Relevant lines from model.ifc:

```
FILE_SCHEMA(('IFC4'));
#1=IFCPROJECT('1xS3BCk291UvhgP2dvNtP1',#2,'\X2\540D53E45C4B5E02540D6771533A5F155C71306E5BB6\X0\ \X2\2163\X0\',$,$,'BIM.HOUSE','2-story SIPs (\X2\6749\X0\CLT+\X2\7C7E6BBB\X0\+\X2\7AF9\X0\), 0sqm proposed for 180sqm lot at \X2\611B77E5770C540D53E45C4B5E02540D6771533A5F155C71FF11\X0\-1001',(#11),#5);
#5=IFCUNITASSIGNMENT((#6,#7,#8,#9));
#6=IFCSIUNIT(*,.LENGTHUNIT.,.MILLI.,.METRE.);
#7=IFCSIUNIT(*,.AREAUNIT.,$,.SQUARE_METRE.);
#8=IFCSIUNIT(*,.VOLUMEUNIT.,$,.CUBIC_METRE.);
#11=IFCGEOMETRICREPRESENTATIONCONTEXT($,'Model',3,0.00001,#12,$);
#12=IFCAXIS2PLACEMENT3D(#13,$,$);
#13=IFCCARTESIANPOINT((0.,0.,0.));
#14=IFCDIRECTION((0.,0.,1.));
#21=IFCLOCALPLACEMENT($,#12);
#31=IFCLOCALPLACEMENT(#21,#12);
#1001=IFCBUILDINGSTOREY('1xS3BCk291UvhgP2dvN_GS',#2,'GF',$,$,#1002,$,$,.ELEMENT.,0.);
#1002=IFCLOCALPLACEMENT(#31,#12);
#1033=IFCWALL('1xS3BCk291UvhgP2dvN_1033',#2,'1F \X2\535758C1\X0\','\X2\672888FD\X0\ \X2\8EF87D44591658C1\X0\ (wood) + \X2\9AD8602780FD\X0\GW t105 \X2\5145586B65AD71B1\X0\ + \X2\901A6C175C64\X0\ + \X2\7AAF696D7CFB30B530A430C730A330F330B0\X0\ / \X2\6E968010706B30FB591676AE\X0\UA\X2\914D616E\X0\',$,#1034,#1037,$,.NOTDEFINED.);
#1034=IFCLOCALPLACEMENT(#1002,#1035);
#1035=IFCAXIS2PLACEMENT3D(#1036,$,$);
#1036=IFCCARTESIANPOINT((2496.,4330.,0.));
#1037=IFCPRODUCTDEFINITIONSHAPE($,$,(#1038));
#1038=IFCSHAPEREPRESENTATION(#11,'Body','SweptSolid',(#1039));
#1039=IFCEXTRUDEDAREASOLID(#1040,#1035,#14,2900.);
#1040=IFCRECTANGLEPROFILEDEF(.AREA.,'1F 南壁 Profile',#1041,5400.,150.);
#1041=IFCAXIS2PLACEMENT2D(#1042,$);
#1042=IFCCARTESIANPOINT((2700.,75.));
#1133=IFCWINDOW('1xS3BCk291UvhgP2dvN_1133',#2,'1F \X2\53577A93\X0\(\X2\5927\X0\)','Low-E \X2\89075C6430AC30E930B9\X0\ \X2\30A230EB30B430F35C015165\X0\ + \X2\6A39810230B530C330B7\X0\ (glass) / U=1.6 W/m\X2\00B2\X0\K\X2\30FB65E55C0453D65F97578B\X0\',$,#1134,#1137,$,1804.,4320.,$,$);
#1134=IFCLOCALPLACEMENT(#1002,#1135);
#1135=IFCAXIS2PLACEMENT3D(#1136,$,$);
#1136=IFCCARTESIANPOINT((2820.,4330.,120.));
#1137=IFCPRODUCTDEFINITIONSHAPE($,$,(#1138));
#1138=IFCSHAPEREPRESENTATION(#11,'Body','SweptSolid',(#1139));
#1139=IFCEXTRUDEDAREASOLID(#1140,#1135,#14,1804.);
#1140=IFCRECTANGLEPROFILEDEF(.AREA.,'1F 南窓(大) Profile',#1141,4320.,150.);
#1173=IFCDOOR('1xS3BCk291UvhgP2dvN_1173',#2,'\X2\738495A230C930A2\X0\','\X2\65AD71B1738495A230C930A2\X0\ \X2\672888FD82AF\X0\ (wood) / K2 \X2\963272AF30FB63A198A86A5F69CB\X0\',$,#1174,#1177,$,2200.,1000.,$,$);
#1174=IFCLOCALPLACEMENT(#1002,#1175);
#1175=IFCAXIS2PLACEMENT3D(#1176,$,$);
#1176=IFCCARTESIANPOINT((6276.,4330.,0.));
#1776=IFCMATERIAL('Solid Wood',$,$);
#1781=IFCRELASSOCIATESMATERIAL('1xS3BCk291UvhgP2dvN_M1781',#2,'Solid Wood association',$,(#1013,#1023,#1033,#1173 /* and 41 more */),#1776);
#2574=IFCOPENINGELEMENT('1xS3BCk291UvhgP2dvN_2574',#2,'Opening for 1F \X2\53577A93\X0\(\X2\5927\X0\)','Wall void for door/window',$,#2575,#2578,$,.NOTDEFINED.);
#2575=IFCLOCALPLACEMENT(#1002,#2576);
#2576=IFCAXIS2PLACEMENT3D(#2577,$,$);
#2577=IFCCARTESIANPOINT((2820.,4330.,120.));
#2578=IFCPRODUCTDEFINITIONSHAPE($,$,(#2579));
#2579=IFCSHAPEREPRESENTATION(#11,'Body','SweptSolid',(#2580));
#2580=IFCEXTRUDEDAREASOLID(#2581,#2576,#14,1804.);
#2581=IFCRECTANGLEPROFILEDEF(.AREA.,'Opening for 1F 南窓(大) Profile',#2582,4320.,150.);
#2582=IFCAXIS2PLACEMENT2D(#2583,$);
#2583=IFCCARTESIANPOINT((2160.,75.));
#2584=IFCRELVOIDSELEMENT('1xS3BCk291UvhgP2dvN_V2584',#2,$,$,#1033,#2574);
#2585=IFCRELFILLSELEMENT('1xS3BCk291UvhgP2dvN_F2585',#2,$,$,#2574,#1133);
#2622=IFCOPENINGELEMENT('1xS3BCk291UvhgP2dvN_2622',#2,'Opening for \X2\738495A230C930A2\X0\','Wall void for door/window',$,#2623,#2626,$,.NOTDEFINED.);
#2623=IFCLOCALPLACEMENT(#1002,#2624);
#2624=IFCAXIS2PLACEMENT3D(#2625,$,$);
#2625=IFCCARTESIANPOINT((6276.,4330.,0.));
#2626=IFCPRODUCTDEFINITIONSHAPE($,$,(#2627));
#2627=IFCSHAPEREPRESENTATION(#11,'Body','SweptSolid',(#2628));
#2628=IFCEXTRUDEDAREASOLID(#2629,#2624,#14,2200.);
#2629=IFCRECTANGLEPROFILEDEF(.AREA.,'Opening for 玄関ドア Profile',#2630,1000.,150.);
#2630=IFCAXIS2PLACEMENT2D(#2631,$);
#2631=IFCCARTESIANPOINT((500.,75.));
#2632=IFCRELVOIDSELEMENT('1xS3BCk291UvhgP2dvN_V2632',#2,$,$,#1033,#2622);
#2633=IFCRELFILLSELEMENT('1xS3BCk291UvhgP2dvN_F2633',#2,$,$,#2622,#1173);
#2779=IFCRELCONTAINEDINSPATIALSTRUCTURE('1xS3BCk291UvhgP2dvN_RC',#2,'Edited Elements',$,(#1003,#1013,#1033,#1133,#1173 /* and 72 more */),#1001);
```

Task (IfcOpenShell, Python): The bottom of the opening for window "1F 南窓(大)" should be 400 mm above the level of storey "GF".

```python
import numpy as np
import ifcopenshell
import ifcopenshell.api.geometry
import ifcopenshell.geom
import ifcopenshell.util.element
import ifcopenshell.util.placement
import ifcopenshell.util.shape
import ifcopenshell.util.unit

model = ifcopenshell.open("model.ifc")
unit_scale = ifcopenshell.util.unit.calculate_unit_scale(model)

window = model.by_guid("1xS3BCk291UvhgP2dvN_1133")
opening = window.FillsVoids[0].RelatingOpeningElement
storey = ifcopenshell.util.element.get_container(window, ifc_class="IfcBuildingStorey")
level = ifcopenshell.util.placement.get_local_placement(storey.ObjectPlacement)[2, 3]

# The opening's origin need not be at the sill, so measure its lowest point.
shape = ifcopenshell.geom.create_shape(ifcopenshell.geom.settings(), opening)
bottom = ifcopenshell.util.shape.get_shape_bottom_elevation(shape, shape.geometry) / unit_scale
dz = level + 400.0 - bottom

shift = np.array([0.0, 0.0, dz])
# The window is not placed relative to its opening, so move both.
for product in (opening, window):
    matrix = ifcopenshell.util.placement.get_local_placement(product.ObjectPlacement)
    matrix[:3, 3] += shift
    ifcopenshell.api.geometry.edit_object_placement(model, product=product, matrix=matrix, is_si=False)

print(f"moved by {dz * unit_scale:+.3f} m")

model.write("model_updated.ifc")
```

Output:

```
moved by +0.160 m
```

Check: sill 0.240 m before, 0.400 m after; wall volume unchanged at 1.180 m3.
